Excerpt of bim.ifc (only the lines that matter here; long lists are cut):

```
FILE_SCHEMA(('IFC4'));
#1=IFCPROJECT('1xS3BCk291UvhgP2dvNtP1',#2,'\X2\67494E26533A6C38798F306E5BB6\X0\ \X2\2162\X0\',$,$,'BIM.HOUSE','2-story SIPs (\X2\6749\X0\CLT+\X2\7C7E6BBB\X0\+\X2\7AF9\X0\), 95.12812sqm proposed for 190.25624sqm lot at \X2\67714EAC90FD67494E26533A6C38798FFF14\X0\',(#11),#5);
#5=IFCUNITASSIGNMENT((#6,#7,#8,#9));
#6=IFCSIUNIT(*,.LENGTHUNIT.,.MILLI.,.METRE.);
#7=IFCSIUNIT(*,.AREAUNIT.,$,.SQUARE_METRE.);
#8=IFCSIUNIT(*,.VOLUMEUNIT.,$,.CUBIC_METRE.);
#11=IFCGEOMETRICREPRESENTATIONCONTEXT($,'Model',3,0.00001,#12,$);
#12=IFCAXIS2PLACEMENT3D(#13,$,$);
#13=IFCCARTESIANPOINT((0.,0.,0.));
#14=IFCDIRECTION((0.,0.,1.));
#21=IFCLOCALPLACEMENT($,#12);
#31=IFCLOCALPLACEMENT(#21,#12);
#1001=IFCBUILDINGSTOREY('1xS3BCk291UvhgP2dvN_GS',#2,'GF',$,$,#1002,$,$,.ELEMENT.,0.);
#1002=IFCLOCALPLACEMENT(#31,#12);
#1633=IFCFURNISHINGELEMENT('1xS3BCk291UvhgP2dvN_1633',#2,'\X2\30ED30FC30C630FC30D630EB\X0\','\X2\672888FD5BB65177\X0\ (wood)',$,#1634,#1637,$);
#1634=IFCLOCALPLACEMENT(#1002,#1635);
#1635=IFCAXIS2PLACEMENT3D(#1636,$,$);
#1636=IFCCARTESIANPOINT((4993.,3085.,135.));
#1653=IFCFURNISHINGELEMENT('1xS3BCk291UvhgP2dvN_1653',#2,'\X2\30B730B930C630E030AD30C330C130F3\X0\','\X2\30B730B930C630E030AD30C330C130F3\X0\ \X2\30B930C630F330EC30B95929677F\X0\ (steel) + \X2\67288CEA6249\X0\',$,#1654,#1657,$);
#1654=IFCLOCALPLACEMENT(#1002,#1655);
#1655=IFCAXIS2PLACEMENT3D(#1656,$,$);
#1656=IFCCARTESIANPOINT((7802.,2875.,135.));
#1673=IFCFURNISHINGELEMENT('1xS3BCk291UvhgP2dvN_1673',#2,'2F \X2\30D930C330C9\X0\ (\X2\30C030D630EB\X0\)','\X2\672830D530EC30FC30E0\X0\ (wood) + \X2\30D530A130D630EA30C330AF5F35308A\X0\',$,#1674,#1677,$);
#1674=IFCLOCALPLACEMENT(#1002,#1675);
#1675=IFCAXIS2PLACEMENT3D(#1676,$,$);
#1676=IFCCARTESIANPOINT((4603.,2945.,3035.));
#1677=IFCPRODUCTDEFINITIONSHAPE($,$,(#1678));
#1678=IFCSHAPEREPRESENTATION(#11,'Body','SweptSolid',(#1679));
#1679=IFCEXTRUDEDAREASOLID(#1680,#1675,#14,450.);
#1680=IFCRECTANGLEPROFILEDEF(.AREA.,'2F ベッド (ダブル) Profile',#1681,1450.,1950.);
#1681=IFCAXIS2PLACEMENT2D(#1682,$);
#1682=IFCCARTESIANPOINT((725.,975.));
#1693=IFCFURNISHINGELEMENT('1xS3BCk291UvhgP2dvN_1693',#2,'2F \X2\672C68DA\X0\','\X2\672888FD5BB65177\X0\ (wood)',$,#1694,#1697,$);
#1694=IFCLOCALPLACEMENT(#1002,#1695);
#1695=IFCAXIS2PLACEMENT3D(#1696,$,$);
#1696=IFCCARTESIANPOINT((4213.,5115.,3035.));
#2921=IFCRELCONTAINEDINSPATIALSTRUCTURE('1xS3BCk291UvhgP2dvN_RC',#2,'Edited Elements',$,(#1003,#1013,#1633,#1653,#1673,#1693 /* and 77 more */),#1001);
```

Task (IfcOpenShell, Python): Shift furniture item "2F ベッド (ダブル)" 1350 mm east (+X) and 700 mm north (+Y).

```python
import ifcopenshell
import ifcopenshell.api.geometry
import ifcopenshell.util.placement
import ifcopenshell.util.unit

model = ifcopenshell.open("bim.ifc")
unit_scale = ifcopenshell.util.unit.calculate_unit_scale(model)

item = model.by_guid("1xS3BCk291UvhgP2dvN_1673")
matrix = ifcopenshell.util.placement.get_local_placement(item.ObjectPlacement)
matrix[0, 3] += 1.35 / unit_scale
matrix[1, 3] += 0.7 / unit_scale
ifcopenshell.api.geometry.edit_object_placement(model, product=item, matrix=matrix, is_si=False)

print(ifcopenshell.util.placement.get_local_placement(item.ObjectPlacement).round(3) + 0.0)

model.write("bim_updated.ifc")
```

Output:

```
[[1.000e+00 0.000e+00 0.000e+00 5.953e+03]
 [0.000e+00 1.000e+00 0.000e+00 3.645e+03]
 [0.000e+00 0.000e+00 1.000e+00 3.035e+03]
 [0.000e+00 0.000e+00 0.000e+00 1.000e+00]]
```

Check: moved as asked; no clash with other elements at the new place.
